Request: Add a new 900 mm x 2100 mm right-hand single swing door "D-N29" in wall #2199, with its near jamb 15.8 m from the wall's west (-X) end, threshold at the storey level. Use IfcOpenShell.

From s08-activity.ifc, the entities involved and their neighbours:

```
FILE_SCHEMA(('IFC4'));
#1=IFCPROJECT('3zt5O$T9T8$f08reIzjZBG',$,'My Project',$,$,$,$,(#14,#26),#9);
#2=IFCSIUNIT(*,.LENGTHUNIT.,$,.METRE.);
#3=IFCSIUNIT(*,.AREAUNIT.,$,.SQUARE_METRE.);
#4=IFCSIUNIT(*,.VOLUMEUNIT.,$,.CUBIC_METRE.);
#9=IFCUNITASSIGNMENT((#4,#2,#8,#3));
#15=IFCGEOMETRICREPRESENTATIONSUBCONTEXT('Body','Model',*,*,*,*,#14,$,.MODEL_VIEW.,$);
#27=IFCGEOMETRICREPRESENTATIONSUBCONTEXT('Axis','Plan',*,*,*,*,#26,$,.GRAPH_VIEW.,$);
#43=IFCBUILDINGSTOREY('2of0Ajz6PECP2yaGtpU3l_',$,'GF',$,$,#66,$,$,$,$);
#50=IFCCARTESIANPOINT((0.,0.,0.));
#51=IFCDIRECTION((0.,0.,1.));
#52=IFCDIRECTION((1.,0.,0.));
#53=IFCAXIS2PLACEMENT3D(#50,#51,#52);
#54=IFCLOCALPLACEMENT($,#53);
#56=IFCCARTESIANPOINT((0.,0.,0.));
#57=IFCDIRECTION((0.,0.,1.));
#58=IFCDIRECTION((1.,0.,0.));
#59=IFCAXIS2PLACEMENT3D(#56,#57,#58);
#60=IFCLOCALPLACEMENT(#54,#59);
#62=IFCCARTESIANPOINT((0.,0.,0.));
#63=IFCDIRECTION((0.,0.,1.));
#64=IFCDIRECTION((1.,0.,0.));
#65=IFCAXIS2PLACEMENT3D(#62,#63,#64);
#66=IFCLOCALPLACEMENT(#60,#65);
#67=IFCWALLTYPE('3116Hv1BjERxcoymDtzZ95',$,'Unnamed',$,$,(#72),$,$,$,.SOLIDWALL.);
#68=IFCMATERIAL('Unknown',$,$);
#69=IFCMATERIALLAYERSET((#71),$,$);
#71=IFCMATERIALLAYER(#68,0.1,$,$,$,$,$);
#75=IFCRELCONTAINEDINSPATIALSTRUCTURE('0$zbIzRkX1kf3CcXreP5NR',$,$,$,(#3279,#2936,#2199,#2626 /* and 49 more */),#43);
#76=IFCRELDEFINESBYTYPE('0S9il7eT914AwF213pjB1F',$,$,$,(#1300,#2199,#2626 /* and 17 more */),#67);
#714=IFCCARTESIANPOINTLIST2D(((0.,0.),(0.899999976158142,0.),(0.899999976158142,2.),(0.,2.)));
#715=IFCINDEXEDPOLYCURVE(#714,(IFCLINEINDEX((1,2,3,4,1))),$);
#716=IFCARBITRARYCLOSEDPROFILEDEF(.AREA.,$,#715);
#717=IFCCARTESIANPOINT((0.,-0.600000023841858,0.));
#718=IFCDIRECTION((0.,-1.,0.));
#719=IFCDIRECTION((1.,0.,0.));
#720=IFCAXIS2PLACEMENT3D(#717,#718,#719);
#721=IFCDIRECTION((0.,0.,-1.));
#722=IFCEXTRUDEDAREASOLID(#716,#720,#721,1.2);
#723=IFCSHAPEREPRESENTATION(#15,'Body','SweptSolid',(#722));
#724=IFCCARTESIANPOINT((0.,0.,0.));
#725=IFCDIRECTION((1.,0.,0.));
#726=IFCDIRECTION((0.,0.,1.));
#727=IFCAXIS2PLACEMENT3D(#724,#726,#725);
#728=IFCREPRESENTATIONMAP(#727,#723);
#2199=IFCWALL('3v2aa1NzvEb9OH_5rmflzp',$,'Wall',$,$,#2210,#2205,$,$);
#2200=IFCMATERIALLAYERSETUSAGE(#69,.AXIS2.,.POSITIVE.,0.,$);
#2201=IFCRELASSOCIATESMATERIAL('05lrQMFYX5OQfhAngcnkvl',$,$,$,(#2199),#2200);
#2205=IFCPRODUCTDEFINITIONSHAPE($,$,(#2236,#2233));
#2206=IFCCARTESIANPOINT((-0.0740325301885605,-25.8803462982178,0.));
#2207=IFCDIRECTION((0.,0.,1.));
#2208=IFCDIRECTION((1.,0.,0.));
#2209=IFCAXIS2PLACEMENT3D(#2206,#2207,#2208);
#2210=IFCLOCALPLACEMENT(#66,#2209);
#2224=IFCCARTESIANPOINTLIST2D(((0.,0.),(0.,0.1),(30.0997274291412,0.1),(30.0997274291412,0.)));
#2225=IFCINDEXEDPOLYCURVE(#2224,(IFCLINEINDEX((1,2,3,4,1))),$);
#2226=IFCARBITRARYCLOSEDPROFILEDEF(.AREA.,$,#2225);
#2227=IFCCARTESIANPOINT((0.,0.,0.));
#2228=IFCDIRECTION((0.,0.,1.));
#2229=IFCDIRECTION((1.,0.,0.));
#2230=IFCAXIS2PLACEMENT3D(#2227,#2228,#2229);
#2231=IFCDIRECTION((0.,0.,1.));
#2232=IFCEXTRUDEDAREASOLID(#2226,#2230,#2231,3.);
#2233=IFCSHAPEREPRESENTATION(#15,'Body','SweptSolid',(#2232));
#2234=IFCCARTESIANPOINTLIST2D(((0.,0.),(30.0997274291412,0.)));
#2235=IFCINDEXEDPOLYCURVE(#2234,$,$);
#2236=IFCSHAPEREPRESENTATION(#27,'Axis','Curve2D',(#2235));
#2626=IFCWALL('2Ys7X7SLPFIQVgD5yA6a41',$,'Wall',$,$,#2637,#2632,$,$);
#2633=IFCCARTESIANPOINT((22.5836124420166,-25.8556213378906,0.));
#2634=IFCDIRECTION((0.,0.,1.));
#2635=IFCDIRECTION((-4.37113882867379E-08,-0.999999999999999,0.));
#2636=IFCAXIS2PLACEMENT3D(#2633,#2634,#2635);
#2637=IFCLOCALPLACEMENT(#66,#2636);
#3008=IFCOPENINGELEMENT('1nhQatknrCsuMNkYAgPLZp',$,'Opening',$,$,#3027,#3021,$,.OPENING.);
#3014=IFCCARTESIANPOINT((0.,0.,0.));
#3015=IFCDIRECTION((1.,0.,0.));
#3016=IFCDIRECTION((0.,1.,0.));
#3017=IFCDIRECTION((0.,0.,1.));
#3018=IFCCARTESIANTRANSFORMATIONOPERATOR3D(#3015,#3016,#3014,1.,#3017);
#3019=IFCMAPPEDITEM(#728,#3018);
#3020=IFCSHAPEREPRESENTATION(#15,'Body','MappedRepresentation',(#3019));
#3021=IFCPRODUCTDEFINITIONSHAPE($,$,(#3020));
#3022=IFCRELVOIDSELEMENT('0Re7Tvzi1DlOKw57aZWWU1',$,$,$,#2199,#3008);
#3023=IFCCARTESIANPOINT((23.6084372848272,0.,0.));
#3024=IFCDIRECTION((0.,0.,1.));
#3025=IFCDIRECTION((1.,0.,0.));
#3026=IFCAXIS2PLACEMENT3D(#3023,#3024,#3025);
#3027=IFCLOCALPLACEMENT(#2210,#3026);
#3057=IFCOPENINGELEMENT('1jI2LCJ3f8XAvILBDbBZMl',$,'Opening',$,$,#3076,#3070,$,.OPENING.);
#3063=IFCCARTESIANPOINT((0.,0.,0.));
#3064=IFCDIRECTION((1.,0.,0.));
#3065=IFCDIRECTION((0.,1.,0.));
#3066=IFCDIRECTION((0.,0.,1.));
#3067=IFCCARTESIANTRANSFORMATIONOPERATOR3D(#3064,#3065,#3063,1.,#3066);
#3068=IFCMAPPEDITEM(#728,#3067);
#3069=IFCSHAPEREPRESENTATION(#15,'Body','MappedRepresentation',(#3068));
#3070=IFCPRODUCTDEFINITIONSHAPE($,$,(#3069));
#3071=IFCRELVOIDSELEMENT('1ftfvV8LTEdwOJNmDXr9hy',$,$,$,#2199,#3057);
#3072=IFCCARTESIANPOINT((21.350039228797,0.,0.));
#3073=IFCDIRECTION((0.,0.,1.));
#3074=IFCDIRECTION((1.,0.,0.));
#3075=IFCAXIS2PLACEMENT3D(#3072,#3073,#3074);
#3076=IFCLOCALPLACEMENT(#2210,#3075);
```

```python
import numpy as np
import ifcopenshell
import ifcopenshell.api.feature
import ifcopenshell.api.geometry
import ifcopenshell.api.root
import ifcopenshell.api.spatial
import ifcopenshell.geom
import ifcopenshell.util.element
import ifcopenshell.util.placement
import ifcopenshell.util.representation
import ifcopenshell.util.shape
import ifcopenshell.util.unit

model = ifcopenshell.open("s08-activity.ifc")
unit_scale = ifcopenshell.util.unit.calculate_unit_scale(model)
settings = ifcopenshell.geom.settings()


def volume(element):
    """Net volume in cubic metres, openings subtracted."""
    shape = ifcopenshell.geom.create_shape(settings, element)
    return ifcopenshell.util.shape.get_volume(shape.geometry)


wall = model.by_id(2199)
storey = ifcopenshell.util.element.get_container(wall, ifc_class="IfcBuildingStorey")
context = ifcopenshell.util.representation.get_context(model, "Model", "Body", "MODEL_VIEW")
before = volume(wall)

width, height, from_end, sill = 0.9, 2.1, 15.8, 0.0  # metres

# The wall runs along its own X axis, and the end named is its -X end.
wall_shape = ifcopenshell.geom.create_shape(settings, wall)
x, y, z = ifcopenshell.util.shape.get_vertices(wall_shape.geometry).T
start = x.min() + from_end
face, thickness = float(y.min()), float(y.max() - y.min())
wall_matrix = ifcopenshell.util.placement.get_local_placement(wall.ObjectPlacement)
level = ifcopenshell.util.placement.get_local_placement(storey.ObjectPlacement)[2, 3]


def in_wall(x, y):
    """Placement at x, y metres in the wall's axes, at sill height."""
    matrix = wall_matrix.copy()
    matrix[:, 3] = wall_matrix @ np.array([x / unit_scale, y / unit_scale, 0.0, 1.0])
    matrix[2, 3] = level + sill / unit_scale
    return matrix


# Opening: a box that overshoots both wall faces by 50 mm.
opening = ifcopenshell.api.root.create_entity(model, ifc_class="IfcOpeningElement", predefined_type="OPENING")
box = ifcopenshell.api.geometry.add_wall_representation(
    model, context=context, length=width, height=height, thickness=thickness + 0.1
)
ifcopenshell.api.geometry.assign_representation(model, product=opening, representation=box)
ifcopenshell.api.geometry.edit_object_placement(model, product=opening, matrix=in_wall(start, face - 0.05), is_si=False)
ifcopenshell.api.feature.add_feature(model, feature=opening, element=wall)

door = ifcopenshell.api.root.create_entity(model, ifc_class="IfcDoor", name="D-N29", predefined_type="DOOR")
door.OverallWidth, door.OverallHeight = width / unit_scale, height / unit_scale
door.OperationType = "SINGLE_SWING_RIGHT"
body = ifcopenshell.api.geometry.add_door_representation(
    model,
    context=context,
    overall_width=door.OverallWidth,
    overall_height=door.OverallHeight,
    operation_type="SINGLE_SWING_RIGHT",
    lining_properties={"LiningDepth": thickness / unit_scale, "ThresholdDepth": thickness / unit_scale},
)
ifcopenshell.api.geometry.assign_representation(model, product=door, representation=body)
ifcopenshell.api.spatial.assign_container(model, products=[door], relating_structure=storey)
ifcopenshell.api.feature.add_filling(model, opening=opening, element=door)

# The lining spans the wall, so the door starts at the wall face.
ifcopenshell.api.geometry.edit_object_placement(model, product=door, matrix=in_wall(start, face), is_si=False)

after = volume(wall)

print(f"wall volume {before:.3f} -> {after:.3f} m3")

model.write("s08-activity_v2.ifc")
```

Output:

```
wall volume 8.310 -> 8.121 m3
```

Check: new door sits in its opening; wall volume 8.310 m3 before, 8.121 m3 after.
